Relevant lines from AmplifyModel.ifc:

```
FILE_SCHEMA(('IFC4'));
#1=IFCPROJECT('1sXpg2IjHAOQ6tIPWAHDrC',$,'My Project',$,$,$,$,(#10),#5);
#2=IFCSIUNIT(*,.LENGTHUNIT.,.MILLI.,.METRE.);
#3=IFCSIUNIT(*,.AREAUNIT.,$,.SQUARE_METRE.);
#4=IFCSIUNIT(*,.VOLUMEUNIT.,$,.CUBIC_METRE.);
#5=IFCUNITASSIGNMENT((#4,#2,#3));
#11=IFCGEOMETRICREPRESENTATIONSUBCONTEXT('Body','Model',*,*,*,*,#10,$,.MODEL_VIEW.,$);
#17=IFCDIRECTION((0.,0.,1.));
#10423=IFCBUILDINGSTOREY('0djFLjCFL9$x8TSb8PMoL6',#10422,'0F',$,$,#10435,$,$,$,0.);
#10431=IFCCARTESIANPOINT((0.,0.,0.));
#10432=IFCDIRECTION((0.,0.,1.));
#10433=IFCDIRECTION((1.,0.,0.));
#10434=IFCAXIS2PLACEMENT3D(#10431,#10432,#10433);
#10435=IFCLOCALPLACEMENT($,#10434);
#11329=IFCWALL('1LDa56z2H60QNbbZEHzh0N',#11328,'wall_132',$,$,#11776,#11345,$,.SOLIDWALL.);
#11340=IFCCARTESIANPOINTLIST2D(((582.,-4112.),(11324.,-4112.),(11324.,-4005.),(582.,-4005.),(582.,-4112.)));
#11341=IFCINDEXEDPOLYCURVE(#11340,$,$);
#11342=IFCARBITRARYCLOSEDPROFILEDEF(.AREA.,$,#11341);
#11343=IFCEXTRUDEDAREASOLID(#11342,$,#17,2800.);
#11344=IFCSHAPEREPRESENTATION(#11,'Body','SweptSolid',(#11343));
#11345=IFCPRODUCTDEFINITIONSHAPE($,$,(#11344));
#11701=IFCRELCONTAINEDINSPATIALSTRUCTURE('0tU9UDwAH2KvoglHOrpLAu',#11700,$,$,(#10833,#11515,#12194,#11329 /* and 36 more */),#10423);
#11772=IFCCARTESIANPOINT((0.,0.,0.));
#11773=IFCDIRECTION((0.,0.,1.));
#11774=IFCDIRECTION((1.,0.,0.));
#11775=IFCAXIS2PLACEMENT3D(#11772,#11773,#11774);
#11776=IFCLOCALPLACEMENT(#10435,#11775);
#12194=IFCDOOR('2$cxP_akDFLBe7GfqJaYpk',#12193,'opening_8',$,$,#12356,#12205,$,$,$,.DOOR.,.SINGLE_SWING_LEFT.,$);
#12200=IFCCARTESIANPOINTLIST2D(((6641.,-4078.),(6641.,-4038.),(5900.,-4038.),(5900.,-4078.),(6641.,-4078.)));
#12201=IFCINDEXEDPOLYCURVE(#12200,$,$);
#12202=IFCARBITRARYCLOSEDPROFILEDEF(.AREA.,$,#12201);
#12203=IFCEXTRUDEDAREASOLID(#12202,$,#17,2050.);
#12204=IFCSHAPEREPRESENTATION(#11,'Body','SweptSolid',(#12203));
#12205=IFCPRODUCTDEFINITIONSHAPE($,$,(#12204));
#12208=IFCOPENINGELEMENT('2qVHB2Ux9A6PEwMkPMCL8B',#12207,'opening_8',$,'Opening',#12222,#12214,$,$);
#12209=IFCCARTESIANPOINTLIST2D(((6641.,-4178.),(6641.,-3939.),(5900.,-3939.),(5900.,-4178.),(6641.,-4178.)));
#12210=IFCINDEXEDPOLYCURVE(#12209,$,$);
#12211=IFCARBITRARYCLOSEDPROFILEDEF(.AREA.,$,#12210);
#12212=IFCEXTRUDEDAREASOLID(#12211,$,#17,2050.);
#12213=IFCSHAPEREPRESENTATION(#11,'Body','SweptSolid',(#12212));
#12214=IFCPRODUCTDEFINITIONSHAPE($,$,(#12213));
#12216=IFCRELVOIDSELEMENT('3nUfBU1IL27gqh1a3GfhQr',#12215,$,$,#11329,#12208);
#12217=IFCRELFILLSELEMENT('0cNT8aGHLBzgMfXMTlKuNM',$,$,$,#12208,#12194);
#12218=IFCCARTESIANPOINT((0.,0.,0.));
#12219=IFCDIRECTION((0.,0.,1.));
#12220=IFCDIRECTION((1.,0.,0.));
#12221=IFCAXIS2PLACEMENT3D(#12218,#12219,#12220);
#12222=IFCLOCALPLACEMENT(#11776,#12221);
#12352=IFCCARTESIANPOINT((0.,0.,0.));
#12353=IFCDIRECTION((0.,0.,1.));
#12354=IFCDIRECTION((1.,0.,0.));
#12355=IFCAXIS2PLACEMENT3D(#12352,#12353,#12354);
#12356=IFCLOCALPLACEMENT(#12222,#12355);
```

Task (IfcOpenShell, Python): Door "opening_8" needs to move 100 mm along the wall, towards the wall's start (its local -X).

```python
import ifcopenshell
import ifcopenshell.api.geometry
import ifcopenshell.util.placement
import ifcopenshell.util.unit

model = ifcopenshell.open("AmplifyModel.ifc")
unit_scale = ifcopenshell.util.unit.calculate_unit_scale(model)

door = model.by_guid("2$cxP_akDFLBe7GfqJaYpk")
opening = door.FillsVoids[0].RelatingOpeningElement
wall = opening.VoidsElements[0].RelatingBuildingElement

wall_matrix = ifcopenshell.util.placement.get_local_placement(wall.ObjectPlacement)
shift = wall_matrix[:3, 0] * -0.1 / unit_scale
before = ifcopenshell.util.placement.get_local_placement(door.ObjectPlacement)[:3, 3].copy()

# The door is placed relative to its opening, so it follows when the opening moves.
matrix = ifcopenshell.util.placement.get_local_placement(opening.ObjectPlacement)
matrix[:3, 3] += shift
ifcopenshell.api.geometry.edit_object_placement(
    model, product=opening, matrix=matrix, is_si=False, should_transform_children=True
)

after = ifcopenshell.util.placement.get_local_placement(door.ObjectPlacement)[:3, 3]
print("door moved by", (after - before).round(3) + 0.0)

model.write("AmplifyModel_rev.ifc")
```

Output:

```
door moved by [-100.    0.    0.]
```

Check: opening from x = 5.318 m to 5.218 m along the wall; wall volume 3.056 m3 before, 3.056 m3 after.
